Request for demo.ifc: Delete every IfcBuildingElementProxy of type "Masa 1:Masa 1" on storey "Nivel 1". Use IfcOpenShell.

First a look at what the model holds.

```python
import ifcopenshell
import ifcopenshell.util.element

model = ifcopenshell.open("demo.ifc")
print(model.schema)
storey = next(s for s in model.by_type("IfcBuildingStorey") if s.Name == "Nivel 1")
proxies = [e for e in ifcopenshell.util.element.get_decomposition(storey) if e.is_a("IfcBuildingElementProxy")]
seen = {}
for e in proxies:
    element_type = ifcopenshell.util.element.get_type(e)
    name = element_type.Name if element_type not in (None, e) else None
    seen[name] = seen.get(name, 0) + 1
for name, count in sorted(seen.items(), key=str):
    print(count, "x", name)
```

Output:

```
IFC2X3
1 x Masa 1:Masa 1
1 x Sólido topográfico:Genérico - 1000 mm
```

```python
import ifcopenshell
import ifcopenshell.api.root
import ifcopenshell.util.element

model = ifcopenshell.open("demo.ifc")

storey = next(s for s in model.by_type("IfcBuildingStorey") if s.Name == "Nivel 1")
proxies = [e for e in ifcopenshell.util.element.get_decomposition(storey) if e.is_a("IfcBuildingElementProxy")]
targets = [e for e in proxies if (t := ifcopenshell.util.element.get_type(e)) not in (None, e) and t.Name == "Masa 1:Masa 1"]

for e in targets:
    ifcopenshell.api.root.remove_product(model, product=e)
print(len(targets), "removed")

model.write("demo-out.ifc")
```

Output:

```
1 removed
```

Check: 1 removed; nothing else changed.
